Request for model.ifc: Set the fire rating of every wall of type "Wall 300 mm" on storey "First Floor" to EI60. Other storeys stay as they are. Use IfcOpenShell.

First a look at what the model holds.

```python
import ifcopenshell
import ifcopenshell.util.element

model = ifcopenshell.open("model.ifc")
print(model.schema)
storey = next(s for s in model.by_type("IfcBuildingStorey") if s.Name == "First Floor")
walls = [e for e in ifcopenshell.util.element.get_decomposition(storey) if e.is_a("IfcWall")]
seen = {}
for e in walls:
    element_type = ifcopenshell.util.element.get_type(e)
    key = (element_type.Name if element_type != e and element_type else None, ifcopenshell.util.element.get_pset(e, "Pset_WallCommon", "FireRating"))
    seen[key] = seen.get(key, 0) + 1
for (name, value), count in sorted(seen.items(), key=str):
    print(count, "x", name, "|", value)
```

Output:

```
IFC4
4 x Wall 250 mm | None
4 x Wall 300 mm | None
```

```python
import ifcopenshell
import ifcopenshell.api.pset
import ifcopenshell.util.element

model = ifcopenshell.open("model.ifc")

storey = next(s for s in model.by_type("IfcBuildingStorey") if s.Name == "First Floor")
walls = [e for e in ifcopenshell.util.element.get_decomposition(storey) if e.is_a("IfcWall")]

count = 0
for e in walls:
    element_type = ifcopenshell.util.element.get_type(e)
    if element_type in (None, e) or element_type.Name != "Wall 300 mm":
        continue
    # add_pset returns the element's existing set when there is one.
    pset = ifcopenshell.api.pset.add_pset(model, product=e, name="Pset_WallCommon")
    ifcopenshell.api.pset.edit_pset(model, pset=pset, properties={"FireRating": "EI60"})
    count += 1

print(count, "walls updated")

model.write("model-out.ifc")
```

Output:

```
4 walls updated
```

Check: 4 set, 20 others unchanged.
